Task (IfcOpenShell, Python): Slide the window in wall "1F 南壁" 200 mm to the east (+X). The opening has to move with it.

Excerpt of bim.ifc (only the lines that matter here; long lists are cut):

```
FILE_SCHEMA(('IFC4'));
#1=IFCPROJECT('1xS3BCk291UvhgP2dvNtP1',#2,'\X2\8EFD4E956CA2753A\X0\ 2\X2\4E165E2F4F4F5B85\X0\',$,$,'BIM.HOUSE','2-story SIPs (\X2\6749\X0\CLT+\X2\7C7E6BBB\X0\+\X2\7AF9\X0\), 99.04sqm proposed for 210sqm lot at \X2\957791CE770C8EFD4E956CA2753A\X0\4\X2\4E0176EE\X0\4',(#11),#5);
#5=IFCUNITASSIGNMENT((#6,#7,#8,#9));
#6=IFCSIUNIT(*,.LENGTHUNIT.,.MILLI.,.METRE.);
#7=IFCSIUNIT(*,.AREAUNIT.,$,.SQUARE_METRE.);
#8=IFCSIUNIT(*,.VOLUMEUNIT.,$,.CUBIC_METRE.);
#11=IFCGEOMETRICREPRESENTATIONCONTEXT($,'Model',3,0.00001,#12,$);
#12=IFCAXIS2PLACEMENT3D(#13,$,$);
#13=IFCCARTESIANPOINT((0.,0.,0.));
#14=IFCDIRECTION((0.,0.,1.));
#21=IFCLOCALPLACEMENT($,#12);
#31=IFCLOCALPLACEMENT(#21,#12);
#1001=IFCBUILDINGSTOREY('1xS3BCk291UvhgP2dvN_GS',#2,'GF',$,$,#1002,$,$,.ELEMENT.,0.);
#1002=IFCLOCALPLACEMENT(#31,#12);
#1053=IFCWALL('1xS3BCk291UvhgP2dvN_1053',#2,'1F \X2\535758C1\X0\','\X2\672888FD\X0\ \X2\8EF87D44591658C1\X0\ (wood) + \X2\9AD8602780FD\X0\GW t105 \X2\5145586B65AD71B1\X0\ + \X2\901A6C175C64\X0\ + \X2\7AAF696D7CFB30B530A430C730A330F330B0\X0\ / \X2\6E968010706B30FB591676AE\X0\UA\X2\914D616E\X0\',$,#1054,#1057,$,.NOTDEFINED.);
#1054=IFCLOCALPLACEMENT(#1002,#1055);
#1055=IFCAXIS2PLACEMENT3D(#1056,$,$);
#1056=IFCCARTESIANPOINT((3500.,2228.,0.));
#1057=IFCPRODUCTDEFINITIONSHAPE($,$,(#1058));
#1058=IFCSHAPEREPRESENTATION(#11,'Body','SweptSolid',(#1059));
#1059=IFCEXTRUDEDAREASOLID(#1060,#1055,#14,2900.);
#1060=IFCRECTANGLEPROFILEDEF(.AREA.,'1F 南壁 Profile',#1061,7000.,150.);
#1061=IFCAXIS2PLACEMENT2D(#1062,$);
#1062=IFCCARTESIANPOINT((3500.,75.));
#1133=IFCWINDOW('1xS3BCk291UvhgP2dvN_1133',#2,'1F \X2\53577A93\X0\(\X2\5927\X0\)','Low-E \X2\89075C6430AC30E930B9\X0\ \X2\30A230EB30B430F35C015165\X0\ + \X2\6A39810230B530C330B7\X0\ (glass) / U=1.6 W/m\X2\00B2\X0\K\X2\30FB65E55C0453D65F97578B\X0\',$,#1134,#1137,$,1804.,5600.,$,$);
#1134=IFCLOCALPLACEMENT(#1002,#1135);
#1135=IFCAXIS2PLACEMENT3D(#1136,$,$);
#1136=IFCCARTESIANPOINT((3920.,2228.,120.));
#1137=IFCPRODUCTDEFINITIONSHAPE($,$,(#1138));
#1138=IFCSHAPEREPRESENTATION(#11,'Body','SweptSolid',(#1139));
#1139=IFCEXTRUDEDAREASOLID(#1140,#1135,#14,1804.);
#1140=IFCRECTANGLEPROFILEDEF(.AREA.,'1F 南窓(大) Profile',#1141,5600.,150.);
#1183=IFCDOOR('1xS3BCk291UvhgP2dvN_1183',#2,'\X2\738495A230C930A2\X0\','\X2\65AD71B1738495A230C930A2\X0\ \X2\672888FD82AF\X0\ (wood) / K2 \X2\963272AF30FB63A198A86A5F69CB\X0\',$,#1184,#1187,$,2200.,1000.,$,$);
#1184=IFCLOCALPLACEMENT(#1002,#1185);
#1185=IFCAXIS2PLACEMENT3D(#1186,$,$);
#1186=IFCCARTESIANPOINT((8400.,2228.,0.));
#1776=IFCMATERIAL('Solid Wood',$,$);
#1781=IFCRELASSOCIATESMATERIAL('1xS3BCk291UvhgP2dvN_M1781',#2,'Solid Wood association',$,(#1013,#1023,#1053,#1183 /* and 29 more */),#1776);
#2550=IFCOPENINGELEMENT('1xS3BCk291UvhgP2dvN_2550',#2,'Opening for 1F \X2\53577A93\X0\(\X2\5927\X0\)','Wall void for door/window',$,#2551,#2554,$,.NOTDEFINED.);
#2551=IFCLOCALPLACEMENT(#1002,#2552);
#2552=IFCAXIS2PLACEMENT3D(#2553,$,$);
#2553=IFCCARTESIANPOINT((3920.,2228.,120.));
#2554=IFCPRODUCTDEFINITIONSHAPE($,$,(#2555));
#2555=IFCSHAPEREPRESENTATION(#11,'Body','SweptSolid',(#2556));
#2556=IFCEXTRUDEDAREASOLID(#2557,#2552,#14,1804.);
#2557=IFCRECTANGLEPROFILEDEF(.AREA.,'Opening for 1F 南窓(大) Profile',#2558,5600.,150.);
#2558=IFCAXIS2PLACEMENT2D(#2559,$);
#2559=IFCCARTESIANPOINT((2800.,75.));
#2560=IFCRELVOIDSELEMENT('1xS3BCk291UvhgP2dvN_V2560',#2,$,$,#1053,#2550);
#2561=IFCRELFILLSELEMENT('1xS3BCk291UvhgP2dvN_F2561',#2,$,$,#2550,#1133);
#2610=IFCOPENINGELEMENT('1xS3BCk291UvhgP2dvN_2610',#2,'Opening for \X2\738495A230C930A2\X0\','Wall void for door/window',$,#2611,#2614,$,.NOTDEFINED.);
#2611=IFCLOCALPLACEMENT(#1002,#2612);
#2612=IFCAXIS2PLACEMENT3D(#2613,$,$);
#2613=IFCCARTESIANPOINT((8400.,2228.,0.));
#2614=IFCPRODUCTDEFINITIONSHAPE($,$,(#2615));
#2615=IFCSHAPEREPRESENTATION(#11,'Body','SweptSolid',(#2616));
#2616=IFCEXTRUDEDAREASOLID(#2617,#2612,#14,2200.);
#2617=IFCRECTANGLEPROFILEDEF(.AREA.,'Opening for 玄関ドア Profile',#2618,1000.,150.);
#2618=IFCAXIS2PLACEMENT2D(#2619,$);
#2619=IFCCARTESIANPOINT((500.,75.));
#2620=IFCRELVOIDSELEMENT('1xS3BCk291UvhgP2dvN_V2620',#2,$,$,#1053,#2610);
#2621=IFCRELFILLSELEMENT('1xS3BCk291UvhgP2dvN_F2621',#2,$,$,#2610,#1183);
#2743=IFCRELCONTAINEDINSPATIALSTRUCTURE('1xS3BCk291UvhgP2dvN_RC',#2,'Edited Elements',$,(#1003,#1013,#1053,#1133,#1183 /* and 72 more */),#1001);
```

```python
import ifcopenshell
import ifcopenshell.api.geometry
import ifcopenshell.util.placement
import ifcopenshell.util.unit

model = ifcopenshell.open("bim.ifc")
unit_scale = ifcopenshell.util.unit.calculate_unit_scale(model)

window = model.by_guid("1xS3BCk291UvhgP2dvN_1133")
opening = window.FillsVoids[0].RelatingOpeningElement
wall = opening.VoidsElements[0].RelatingBuildingElement

wall_matrix = ifcopenshell.util.placement.get_local_placement(wall.ObjectPlacement)
shift = wall_matrix[:3, 0] * 0.2 / unit_scale
before = ifcopenshell.util.placement.get_local_placement(window.ObjectPlacement)[:3, 3].copy()

# The window is not placed relative to its opening, so move both.
for product in (opening, window):
    matrix = ifcopenshell.util.placement.get_local_placement(product.ObjectPlacement)
    matrix[:3, 3] += shift
    ifcopenshell.api.geometry.edit_object_placement(model, product=product, matrix=matrix, is_si=False)

after = ifcopenshell.util.placement.get_local_placement(window.ObjectPlacement)[:3, 3]
print("window moved by", (after - before).round(3) + 0.0)

model.write("bim_rev.ifc")
```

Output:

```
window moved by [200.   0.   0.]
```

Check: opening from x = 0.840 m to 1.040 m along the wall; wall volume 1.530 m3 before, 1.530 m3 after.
